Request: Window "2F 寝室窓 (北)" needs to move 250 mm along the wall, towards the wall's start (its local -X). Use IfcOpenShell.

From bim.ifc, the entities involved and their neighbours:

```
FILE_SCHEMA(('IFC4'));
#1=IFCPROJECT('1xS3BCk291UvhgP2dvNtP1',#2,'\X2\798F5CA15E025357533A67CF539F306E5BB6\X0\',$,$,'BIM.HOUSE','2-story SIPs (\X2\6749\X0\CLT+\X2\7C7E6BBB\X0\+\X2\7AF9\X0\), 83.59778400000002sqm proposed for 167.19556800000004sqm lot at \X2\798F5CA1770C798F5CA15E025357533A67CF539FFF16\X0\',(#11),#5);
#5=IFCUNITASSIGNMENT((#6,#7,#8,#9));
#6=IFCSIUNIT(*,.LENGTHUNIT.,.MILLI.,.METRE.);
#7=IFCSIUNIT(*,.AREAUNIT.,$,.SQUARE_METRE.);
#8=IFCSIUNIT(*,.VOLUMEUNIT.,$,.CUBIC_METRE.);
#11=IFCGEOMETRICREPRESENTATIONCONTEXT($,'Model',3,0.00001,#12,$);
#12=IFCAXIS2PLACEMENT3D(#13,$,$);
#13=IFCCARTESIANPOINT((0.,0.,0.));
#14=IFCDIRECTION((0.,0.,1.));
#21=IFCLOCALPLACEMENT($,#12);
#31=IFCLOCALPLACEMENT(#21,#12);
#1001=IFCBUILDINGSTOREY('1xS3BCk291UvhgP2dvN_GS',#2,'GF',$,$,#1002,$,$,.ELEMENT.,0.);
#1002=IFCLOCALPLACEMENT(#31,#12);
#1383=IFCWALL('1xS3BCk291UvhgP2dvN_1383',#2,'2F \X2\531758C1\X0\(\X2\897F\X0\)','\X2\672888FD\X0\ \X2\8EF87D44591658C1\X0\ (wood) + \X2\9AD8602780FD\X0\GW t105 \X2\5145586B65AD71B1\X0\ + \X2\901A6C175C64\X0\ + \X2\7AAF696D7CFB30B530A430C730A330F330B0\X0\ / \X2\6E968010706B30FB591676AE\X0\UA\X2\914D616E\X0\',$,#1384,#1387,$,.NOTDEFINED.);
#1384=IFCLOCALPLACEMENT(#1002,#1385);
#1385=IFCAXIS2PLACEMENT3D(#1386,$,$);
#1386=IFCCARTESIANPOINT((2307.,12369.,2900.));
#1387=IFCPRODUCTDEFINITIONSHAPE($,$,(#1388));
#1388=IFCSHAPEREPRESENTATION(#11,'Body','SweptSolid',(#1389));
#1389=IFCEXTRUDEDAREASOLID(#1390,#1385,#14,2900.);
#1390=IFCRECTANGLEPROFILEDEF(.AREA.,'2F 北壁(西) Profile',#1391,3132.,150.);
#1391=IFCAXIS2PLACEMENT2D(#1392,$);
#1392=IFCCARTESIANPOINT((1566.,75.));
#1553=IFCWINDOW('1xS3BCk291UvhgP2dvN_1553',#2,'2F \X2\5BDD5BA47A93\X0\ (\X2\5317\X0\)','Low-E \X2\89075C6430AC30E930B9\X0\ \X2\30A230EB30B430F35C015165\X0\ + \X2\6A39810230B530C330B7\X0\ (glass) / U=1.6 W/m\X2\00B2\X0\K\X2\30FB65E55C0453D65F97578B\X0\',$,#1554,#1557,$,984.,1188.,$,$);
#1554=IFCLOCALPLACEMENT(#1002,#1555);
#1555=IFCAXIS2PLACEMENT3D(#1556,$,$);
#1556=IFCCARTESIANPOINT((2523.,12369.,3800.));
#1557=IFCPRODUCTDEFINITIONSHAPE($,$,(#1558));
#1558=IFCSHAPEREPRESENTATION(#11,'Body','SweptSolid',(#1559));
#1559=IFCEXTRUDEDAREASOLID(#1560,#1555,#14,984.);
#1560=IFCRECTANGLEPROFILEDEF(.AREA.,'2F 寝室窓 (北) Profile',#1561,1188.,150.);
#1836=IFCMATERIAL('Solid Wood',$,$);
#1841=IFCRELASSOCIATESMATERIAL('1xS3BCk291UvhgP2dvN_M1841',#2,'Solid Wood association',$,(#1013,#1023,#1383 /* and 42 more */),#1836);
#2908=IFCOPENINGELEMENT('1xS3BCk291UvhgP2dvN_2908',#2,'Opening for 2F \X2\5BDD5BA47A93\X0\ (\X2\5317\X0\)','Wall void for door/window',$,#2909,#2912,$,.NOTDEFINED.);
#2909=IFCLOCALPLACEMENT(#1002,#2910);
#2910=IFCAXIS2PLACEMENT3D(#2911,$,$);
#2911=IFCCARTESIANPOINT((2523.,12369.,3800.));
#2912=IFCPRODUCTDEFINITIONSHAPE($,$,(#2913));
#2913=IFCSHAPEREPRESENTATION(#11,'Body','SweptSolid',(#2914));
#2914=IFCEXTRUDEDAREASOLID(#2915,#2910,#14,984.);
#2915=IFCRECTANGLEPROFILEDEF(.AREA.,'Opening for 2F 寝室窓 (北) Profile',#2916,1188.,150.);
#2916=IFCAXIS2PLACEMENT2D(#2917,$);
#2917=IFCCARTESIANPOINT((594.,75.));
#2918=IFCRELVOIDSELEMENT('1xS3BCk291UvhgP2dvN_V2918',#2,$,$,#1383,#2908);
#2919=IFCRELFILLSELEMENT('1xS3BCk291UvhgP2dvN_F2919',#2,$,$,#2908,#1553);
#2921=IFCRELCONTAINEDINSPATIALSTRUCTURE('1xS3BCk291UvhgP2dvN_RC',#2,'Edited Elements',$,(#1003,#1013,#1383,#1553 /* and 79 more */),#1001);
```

```python
import ifcopenshell
import ifcopenshell.api.geometry
import ifcopenshell.util.placement
import ifcopenshell.util.unit

model = ifcopenshell.open("bim.ifc")
unit_scale = ifcopenshell.util.unit.calculate_unit_scale(model)

window = model.by_guid("1xS3BCk291UvhgP2dvN_1553")
opening = window.FillsVoids[0].RelatingOpeningElement
wall = opening.VoidsElements[0].RelatingBuildingElement

wall_matrix = ifcopenshell.util.placement.get_local_placement(wall.ObjectPlacement)
shift = wall_matrix[:3, 0] * -0.25 / unit_scale
before = ifcopenshell.util.placement.get_local_placement(window.ObjectPlacement)[:3, 3].copy()

# The window is not placed relative to its opening, so move both.
for product in (opening, window):
    matrix = ifcopenshell.util.placement.get_local_placement(product.ObjectPlacement)
    matrix[:3, 3] += shift
    ifcopenshell.api.geometry.edit_object_placement(model, product=product, matrix=matrix, is_si=False)

after = ifcopenshell.util.placement.get_local_placement(window.ObjectPlacement)[:3, 3]
print("window moved by", (after - before).round(3) + 0.0)

model.write("bim_edited.ifc")
```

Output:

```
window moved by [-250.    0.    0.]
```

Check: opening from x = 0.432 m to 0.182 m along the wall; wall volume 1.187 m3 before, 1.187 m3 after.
